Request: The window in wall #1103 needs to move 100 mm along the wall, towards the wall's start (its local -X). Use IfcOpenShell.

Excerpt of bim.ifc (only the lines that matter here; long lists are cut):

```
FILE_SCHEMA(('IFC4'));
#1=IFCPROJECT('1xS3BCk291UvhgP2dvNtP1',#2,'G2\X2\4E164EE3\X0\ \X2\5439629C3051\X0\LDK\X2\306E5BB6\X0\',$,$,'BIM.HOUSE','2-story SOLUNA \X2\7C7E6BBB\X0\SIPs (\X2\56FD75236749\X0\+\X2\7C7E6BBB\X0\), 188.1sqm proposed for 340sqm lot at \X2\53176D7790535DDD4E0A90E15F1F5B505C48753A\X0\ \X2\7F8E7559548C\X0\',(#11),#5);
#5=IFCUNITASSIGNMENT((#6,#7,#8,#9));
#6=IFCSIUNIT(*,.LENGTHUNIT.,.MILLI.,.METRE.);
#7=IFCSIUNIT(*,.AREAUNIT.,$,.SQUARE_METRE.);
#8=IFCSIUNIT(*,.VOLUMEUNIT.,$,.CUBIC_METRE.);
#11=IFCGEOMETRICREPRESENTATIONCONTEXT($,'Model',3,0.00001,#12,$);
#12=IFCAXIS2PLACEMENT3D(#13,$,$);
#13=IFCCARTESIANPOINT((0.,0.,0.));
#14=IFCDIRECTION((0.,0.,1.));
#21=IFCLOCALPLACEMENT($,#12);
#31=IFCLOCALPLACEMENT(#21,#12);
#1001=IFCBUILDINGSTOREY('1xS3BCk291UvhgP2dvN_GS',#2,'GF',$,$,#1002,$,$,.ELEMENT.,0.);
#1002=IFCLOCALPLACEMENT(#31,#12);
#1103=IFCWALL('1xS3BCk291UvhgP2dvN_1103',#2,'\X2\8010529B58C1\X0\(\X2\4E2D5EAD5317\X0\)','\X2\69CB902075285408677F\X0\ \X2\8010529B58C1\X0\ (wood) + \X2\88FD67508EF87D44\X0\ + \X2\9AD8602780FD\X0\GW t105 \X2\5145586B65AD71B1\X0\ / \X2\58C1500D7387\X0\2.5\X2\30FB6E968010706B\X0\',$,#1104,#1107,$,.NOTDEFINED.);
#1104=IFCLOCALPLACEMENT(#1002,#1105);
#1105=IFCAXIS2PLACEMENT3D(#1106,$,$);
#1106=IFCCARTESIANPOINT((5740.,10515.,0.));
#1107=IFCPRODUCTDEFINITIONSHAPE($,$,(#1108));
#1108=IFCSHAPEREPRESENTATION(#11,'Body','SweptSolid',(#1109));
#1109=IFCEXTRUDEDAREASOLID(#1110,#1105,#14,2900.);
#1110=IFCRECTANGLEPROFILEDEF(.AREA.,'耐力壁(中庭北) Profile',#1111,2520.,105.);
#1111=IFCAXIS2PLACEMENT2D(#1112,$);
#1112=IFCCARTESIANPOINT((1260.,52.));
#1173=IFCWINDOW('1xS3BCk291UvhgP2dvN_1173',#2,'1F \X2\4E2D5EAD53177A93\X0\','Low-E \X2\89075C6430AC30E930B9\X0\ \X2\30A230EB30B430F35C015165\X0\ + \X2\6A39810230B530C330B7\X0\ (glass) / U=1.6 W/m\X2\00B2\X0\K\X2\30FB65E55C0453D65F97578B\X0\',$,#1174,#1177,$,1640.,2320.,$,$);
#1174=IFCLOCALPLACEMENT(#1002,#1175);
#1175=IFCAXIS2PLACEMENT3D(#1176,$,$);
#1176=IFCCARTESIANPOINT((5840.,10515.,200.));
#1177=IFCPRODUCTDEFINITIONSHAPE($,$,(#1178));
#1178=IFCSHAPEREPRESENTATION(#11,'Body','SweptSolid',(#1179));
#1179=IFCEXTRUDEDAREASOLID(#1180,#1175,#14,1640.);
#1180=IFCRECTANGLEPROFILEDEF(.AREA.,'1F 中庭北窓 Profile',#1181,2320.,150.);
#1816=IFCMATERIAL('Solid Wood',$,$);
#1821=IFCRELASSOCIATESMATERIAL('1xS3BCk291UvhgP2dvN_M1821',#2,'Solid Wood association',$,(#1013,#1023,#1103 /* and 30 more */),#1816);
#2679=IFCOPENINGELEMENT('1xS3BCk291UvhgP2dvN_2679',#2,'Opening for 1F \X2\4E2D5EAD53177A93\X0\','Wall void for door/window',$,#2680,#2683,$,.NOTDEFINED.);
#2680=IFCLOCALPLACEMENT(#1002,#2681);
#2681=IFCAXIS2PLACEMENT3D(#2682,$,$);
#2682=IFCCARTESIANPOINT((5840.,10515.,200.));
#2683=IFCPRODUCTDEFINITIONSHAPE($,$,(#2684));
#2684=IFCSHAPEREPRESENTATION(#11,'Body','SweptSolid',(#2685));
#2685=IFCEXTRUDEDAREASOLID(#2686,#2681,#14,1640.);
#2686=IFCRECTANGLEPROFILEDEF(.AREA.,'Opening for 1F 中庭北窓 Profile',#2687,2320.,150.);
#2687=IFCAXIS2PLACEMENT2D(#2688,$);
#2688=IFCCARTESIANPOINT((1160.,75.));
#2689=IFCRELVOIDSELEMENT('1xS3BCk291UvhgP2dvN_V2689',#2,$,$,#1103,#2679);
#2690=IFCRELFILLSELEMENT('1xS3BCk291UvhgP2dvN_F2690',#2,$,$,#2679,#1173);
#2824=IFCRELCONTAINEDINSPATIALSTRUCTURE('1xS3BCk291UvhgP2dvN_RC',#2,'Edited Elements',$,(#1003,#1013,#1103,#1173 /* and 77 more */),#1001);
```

```python
import ifcopenshell
import ifcopenshell.api.geometry
import ifcopenshell.util.placement

model = ifcopenshell.open("bim.ifc")

window = model.by_guid("1xS3BCk291UvhgP2dvN_1173")
opening = window.FillsVoids[0].RelatingOpeningElement
wall = opening.VoidsElements[0].RelatingBuildingElement

wall_matrix = ifcopenshell.util.placement.get_local_placement(wall.ObjectPlacement)
shift = wall_matrix[:3, 0] * -100.0
before = ifcopenshell.util.placement.get_local_placement(window.ObjectPlacement)[:3, 3].copy()

# The window is not placed relative to its opening, so move both.
for product in (opening, window):
    matrix = ifcopenshell.util.placement.get_local_placement(product.ObjectPlacement)
    matrix[:3, 3] += shift
    ifcopenshell.api.geometry.edit_object_placement(model, product=product, matrix=matrix, is_si=False)

after = ifcopenshell.util.placement.get_local_placement(window.ObjectPlacement)[:3, 3]
print("window moved by", (after - before).round(3) + 0.0)

model.write("bim_v2.ifc")
```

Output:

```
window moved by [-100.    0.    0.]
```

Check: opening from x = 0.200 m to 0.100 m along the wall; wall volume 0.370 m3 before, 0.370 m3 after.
